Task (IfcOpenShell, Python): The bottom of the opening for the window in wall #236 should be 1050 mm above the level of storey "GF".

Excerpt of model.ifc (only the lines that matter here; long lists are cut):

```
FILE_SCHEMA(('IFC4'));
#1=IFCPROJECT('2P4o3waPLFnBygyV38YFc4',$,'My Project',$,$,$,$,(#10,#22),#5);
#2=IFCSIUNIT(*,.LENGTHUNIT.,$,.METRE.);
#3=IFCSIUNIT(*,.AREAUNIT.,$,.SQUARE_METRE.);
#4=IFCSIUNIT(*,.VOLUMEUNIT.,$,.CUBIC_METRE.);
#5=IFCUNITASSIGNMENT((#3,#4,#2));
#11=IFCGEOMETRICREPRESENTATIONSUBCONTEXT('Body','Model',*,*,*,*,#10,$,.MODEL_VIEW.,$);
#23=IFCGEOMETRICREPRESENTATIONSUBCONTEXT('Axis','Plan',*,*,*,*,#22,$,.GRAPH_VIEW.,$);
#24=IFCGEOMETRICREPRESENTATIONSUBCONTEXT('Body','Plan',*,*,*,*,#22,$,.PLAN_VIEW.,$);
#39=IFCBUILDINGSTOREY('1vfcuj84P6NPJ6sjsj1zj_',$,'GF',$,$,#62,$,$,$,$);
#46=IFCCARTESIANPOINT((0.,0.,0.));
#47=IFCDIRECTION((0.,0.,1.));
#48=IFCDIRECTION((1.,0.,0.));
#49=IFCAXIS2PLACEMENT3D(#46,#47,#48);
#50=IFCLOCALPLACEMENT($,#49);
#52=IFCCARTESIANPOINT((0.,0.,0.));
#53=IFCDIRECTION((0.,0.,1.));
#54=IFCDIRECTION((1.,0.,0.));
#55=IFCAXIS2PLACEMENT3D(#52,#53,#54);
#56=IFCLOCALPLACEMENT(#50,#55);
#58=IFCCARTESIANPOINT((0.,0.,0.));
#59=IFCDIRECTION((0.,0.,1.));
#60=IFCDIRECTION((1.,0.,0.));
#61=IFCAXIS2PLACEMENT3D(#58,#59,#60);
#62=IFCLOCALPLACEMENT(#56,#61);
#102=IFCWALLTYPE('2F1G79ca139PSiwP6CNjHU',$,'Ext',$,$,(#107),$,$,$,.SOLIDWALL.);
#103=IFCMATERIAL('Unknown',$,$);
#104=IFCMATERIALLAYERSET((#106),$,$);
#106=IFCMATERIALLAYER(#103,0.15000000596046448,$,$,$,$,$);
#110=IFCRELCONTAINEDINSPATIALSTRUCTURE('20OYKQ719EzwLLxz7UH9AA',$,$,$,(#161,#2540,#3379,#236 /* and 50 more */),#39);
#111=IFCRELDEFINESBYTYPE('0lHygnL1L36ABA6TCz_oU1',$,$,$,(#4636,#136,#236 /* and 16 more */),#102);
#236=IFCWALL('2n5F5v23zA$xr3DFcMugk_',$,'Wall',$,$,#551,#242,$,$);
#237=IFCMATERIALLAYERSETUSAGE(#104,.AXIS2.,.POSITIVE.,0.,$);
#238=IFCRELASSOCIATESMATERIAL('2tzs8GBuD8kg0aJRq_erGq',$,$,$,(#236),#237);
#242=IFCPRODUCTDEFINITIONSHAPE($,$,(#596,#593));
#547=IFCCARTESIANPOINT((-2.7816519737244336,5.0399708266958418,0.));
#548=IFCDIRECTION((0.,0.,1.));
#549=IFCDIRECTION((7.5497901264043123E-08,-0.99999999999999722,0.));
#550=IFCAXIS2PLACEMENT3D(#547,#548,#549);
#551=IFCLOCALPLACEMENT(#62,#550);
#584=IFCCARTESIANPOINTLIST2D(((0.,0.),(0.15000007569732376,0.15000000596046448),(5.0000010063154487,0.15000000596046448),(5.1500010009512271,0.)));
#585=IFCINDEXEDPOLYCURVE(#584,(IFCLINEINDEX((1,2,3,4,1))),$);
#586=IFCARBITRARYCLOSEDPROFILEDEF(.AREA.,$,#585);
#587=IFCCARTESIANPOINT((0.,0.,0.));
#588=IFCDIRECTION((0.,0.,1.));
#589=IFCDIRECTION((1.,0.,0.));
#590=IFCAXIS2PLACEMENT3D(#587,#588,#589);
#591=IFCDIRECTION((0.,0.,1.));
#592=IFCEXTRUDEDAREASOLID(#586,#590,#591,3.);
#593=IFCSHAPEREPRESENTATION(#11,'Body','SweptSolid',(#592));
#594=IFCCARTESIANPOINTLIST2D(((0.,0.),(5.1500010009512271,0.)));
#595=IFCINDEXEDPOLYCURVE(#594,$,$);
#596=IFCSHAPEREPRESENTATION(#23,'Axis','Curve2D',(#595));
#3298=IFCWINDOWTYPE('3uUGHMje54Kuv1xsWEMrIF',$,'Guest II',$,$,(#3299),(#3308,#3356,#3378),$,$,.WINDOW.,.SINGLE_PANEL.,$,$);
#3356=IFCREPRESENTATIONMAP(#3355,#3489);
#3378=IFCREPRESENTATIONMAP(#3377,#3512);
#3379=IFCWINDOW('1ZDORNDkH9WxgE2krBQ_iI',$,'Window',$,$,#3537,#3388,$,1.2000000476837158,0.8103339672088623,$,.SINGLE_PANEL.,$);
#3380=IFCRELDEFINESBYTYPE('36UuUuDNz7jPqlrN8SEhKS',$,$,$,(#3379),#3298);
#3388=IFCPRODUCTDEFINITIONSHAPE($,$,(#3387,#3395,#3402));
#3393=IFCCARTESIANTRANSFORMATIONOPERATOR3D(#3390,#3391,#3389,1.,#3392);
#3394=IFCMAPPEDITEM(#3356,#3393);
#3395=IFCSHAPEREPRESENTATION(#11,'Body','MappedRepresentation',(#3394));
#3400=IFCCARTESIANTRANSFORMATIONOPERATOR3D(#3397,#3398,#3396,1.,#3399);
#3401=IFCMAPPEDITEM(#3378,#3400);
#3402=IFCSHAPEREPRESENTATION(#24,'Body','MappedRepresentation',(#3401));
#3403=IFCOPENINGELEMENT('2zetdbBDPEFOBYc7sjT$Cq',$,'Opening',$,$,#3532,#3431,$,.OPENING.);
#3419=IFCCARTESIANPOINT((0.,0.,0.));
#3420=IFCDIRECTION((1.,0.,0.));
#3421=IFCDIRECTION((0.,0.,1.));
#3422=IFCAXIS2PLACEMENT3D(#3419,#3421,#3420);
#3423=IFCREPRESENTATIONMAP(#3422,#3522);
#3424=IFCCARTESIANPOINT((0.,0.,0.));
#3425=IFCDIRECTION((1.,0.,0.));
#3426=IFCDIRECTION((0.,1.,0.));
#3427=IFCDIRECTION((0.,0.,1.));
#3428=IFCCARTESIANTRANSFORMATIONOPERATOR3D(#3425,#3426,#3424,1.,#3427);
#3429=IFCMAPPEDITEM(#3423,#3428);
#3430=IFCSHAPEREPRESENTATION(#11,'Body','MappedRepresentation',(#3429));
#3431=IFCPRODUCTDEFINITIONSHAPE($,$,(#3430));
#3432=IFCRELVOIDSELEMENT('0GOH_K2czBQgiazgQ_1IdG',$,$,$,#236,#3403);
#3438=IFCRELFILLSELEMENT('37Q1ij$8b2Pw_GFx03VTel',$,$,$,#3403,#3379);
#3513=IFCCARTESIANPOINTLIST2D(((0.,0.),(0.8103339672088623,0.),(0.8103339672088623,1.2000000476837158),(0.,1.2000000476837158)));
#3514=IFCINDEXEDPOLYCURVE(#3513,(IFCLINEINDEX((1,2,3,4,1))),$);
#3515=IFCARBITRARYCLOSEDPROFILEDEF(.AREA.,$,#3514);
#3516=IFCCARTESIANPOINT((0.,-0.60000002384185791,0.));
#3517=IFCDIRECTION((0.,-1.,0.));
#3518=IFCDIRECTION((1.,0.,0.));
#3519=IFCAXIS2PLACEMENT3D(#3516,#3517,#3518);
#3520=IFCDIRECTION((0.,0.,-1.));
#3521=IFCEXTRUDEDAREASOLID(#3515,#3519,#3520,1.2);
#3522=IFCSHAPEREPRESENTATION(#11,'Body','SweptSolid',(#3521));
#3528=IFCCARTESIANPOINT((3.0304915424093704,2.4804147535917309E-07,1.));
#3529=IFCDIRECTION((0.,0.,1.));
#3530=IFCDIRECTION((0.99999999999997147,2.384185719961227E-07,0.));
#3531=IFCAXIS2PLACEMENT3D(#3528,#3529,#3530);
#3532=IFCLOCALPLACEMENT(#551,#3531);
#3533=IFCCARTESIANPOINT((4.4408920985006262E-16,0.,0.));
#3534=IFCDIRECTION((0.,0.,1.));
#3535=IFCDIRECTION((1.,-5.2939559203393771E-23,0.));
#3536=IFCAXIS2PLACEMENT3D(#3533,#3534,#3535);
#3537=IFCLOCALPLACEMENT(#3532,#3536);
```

```python
import numpy as np
import ifcopenshell
import ifcopenshell.api.geometry
import ifcopenshell.geom
import ifcopenshell.util.element
import ifcopenshell.util.placement
import ifcopenshell.util.shape
import ifcopenshell.util.unit

model = ifcopenshell.open("model.ifc")
unit_scale = ifcopenshell.util.unit.calculate_unit_scale(model)

window = model.by_id(3379)
opening = window.FillsVoids[0].RelatingOpeningElement
storey = ifcopenshell.util.element.get_container(window, ifc_class="IfcBuildingStorey")
level = ifcopenshell.util.placement.get_local_placement(storey.ObjectPlacement)[2, 3]

# The opening's origin need not be at the sill, so measure its lowest point.
shape = ifcopenshell.geom.create_shape(ifcopenshell.geom.settings(), opening)
bottom = ifcopenshell.util.shape.get_shape_bottom_elevation(shape, shape.geometry) / unit_scale
dz = level + 1.05 - bottom

shift = np.array([0.0, 0.0, dz])
# The window is placed relative to its opening, so it follows when the opening moves.
matrix = ifcopenshell.util.placement.get_local_placement(opening.ObjectPlacement)
matrix[:3, 3] += shift
ifcopenshell.api.geometry.edit_object_placement(
    model, product=opening, matrix=matrix, is_si=False, should_transform_children=True
)

print(f"moved by {dz * unit_scale:+.3f} m")

model.write("model_rev.ifc")
```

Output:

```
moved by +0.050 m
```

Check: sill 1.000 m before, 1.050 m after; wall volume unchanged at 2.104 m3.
